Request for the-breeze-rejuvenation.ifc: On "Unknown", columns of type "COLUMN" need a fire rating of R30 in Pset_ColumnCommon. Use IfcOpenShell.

First a look at what the model holds.

```python
import ifcopenshell
import ifcopenshell.util.element

model = ifcopenshell.open("the-breeze-rejuvenation.ifc")
print(model.schema)
storey = next(s for s in model.by_type("IfcBuildingStorey") if s.Name == "Unknown")
columns = [e for e in ifcopenshell.util.element.get_decomposition(storey) if e.is_a("IfcColumn")]
seen = {}
for e in columns:
    element_type = ifcopenshell.util.element.get_type(e)
    key = (element_type.Name if element_type != e and element_type else None, ifcopenshell.util.element.get_pset(e, "Pset_ColumnCommon", "FireRating"))
    seen[key] = seen.get(key, 0) + 1
for (name, value), count in sorted(seen.items(), key=str):
    print(count, "x", name, "|", value)
```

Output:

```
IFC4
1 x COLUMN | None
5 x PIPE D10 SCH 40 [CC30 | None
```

```python
import ifcopenshell
import ifcopenshell.api.pset
import ifcopenshell.util.element

model = ifcopenshell.open("the-breeze-rejuvenation.ifc")

storey = next(s for s in model.by_type("IfcBuildingStorey") if s.Name == "Unknown")
columns = [e for e in ifcopenshell.util.element.get_decomposition(storey) if e.is_a("IfcColumn")]

count = 0
for e in columns:
    element_type = ifcopenshell.util.element.get_type(e)
    if element_type in (None, e) or element_type.Name != "COLUMN":
        continue
    found = ifcopenshell.util.element.get_pset(e, "Pset_ColumnCommon", should_inherit=False)
    if found:
        pset = model.by_id(found["id"])
        if len(ifcopenshell.util.element.get_elements_by_pset(pset)) > 1:
            pset = ifcopenshell.api.pset.unshare_pset(model, products=[e], pset=pset)[0]
    else:
        pset = ifcopenshell.api.pset.add_pset(model, product=e, name="Pset_ColumnCommon")
    ifcopenshell.api.pset.edit_pset(model, pset=pset, properties={"FireRating": "R30"})
    count += 1

print(count, "columns updated")

model.write("the-breeze-rejuvenation_v2.ifc")
```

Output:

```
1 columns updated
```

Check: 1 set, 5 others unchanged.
